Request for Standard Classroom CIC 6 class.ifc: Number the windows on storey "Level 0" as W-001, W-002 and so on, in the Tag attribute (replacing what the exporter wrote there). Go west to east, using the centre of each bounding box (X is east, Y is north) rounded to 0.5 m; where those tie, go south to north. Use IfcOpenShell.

First a look at what the model holds.

```python
import ifcopenshell
import ifcopenshell.util.element
import ifcopenshell.util.placement

model = ifcopenshell.open("Standard Classroom CIC 6 class.ifc")
print(model.schema)
storey = next(s for s in model.by_type("IfcBuildingStorey") if s.Name == "Level 0")
windows = [e for e in ifcopenshell.util.element.get_decomposition(storey) if e.is_a("IfcWindow")]
for e in sorted(windows, key=lambda e: e.id()):
    origin = ifcopenshell.util.placement.get_local_placement(e.ObjectPlacement)[:3, 3]
    print(e.id(), e.Tag, e.Name, origin.round(2) + 0.0, sep=" | ")
```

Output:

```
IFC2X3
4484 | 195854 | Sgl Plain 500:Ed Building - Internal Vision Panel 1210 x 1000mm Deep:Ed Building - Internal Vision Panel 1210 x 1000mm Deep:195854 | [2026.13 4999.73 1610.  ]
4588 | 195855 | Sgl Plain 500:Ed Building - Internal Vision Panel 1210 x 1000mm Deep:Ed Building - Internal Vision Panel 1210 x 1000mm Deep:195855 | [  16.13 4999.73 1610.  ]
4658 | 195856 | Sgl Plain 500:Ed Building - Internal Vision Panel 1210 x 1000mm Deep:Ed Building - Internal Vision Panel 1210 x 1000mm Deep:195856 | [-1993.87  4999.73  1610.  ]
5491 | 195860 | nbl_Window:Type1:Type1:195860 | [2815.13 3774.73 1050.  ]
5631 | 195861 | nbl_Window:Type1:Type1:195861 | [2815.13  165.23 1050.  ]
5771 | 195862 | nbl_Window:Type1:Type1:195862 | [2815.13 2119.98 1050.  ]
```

```python
import ifcopenshell
import ifcopenshell.geom
import ifcopenshell.util.element
import ifcopenshell.util.shape

model = ifcopenshell.open("Standard Classroom CIC 6 class.ifc")
settings = ifcopenshell.geom.settings()
settings.set("use-world-coords", True)


def centre(element):
    shape = ifcopenshell.geom.create_shape(settings, element)
    return ifcopenshell.util.shape.get_bbox_centroid(shape.geometry)


storey = next(s for s in model.by_type("IfcBuildingStorey") if s.Name == "Level 0")
windows = [e for e in ifcopenshell.util.element.get_decomposition(storey) if e.is_a("IfcWindow")]

# Insertion points can sit at a corner or the storey origin, so sort by the geometry (in metres).
centres = {e: centre(e) for e in windows}
windows.sort(key=lambda e: (round(centres[e][0] / 0.5), centres[e][1]))

for i, e in enumerate(windows, start=1):
    number = f"W-0{i:02d}"
    e.Tag = number
    print(e.id(), number)

model.write("Standard Classroom CIC 6 class_v2.ifc")
```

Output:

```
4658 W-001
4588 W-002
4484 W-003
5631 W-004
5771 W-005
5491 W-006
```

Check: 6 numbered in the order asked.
